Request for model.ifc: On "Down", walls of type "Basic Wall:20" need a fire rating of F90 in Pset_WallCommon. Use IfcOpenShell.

First a look at what the model holds.

```python
import ifcopenshell
import ifcopenshell.util.element

model = ifcopenshell.open("model.ifc")
print(model.schema)
storey = next(s for s in model.by_type("IfcBuildingStorey") if s.Name == "Down")
walls = [e for e in ifcopenshell.util.element.get_decomposition(storey) if e.is_a("IfcWall")]
seen = {}
for e in walls:
    element_type = ifcopenshell.util.element.get_type(e)
    key = (element_type.Name if element_type != e and element_type else None, ifcopenshell.util.element.get_pset(e, "Pset_WallCommon", "FireRating"))
    seen[key] = seen.get(key, 0) + 1
for (name, value), count in sorted(seen.items(), key=str):
    print(count, "x", name, "|", value)
```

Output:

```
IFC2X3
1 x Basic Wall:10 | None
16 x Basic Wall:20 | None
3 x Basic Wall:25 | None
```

```python
import ifcopenshell
import ifcopenshell.api.pset
import ifcopenshell.util.element

model = ifcopenshell.open("model.ifc")

storey = next(s for s in model.by_type("IfcBuildingStorey") if s.Name == "Down")
walls = [e for e in ifcopenshell.util.element.get_decomposition(storey) if e.is_a("IfcWall")]

count = 0
for e in walls:
    element_type = ifcopenshell.util.element.get_type(e)
    if element_type in (None, e) or element_type.Name != "Basic Wall:20":
        continue
    # add_pset returns the element's existing set when there is one.
    pset = ifcopenshell.api.pset.add_pset(model, product=e, name="Pset_WallCommon")
    ifcopenshell.api.pset.edit_pset(model, pset=pset, properties={"FireRating": "F90"})
    count += 1

print(count, "walls updated")

model.write("model_edited.ifc")
```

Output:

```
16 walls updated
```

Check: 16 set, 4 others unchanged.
